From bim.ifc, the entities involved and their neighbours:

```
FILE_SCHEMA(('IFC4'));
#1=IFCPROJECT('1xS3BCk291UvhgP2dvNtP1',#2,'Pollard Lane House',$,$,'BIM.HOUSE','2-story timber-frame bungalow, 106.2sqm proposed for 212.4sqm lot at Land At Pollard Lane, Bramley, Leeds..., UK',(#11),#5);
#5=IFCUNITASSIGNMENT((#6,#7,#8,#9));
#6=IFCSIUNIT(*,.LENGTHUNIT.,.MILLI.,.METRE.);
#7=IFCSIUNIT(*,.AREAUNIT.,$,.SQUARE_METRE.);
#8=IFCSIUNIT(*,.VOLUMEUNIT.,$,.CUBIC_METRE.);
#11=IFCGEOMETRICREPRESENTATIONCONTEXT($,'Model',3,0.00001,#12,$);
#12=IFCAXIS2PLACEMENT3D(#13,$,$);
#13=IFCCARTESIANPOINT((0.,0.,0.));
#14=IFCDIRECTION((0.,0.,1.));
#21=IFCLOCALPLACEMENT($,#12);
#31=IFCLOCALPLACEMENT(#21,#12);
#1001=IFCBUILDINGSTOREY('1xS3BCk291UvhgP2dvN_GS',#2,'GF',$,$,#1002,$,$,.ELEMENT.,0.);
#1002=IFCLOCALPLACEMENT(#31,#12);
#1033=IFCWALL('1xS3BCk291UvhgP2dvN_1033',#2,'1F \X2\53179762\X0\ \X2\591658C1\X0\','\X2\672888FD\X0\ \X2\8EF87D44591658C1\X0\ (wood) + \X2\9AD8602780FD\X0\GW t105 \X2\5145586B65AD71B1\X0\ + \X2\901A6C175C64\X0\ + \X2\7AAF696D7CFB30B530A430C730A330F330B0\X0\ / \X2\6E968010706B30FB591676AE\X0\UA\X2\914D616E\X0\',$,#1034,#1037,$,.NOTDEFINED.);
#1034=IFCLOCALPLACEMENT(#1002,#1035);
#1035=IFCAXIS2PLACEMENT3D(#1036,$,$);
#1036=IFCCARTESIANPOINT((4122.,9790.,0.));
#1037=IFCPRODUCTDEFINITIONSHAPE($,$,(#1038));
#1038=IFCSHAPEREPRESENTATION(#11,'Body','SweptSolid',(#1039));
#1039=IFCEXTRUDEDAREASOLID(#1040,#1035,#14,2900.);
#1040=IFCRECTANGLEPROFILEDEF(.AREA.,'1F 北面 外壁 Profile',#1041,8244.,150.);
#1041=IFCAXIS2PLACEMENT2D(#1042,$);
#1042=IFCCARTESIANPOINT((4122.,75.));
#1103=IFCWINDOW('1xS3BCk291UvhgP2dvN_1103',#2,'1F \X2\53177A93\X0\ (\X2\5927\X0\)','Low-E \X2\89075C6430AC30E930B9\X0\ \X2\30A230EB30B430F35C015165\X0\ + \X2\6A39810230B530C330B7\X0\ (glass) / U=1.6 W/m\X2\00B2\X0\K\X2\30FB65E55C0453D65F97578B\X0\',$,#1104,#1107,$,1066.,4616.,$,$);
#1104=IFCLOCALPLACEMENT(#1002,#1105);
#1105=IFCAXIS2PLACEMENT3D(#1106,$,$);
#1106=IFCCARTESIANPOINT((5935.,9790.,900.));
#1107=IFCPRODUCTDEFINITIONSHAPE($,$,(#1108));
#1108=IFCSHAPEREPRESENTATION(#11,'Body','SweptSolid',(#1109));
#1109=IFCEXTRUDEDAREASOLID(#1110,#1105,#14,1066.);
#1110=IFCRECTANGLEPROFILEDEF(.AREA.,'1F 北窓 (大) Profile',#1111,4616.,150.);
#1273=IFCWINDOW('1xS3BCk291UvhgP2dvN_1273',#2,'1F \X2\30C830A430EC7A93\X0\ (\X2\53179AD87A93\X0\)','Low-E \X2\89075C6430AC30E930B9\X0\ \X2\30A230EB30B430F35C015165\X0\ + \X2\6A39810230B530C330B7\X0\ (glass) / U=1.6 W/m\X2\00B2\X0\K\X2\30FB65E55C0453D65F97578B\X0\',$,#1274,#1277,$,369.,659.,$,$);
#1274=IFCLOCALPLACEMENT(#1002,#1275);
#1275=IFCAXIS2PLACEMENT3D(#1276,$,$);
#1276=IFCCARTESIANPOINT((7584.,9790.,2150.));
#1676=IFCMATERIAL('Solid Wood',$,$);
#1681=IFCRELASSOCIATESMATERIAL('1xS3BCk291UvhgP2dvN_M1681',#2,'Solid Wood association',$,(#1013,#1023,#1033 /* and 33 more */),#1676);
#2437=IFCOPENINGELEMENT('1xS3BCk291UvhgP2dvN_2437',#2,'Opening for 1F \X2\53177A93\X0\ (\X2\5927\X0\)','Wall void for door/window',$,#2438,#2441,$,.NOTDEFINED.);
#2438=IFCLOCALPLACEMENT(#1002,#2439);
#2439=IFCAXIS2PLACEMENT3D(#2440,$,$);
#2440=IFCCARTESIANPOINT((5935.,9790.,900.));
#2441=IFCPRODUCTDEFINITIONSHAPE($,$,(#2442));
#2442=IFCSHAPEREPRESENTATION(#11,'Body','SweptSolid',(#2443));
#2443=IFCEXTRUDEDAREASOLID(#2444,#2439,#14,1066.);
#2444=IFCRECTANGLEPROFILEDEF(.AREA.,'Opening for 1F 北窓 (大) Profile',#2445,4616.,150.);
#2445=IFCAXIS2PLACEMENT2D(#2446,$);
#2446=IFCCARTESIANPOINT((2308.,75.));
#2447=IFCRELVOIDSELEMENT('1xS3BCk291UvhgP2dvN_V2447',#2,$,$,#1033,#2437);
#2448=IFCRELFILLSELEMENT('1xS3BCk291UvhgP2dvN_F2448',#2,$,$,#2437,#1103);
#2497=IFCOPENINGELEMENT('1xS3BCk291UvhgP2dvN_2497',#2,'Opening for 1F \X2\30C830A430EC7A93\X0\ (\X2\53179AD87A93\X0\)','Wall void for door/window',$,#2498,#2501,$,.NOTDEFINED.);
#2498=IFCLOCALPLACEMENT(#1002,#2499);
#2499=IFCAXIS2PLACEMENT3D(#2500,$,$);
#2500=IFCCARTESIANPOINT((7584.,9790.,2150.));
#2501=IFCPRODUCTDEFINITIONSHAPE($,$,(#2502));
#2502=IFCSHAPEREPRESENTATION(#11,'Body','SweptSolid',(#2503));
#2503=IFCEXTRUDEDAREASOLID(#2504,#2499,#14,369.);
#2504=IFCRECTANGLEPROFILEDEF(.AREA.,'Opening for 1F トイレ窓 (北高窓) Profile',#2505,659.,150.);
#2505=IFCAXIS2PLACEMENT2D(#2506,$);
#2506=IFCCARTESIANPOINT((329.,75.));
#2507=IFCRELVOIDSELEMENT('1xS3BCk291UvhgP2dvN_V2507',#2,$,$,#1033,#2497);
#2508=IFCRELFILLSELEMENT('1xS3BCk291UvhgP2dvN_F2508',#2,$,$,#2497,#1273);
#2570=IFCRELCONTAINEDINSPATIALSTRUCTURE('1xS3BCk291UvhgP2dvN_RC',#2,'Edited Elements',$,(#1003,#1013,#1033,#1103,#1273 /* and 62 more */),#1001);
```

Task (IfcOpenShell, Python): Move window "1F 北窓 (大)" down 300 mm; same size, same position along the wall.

```python
import numpy as np
import ifcopenshell
import ifcopenshell.api.geometry
import ifcopenshell.util.placement
import ifcopenshell.util.unit

model = ifcopenshell.open("bim.ifc")
unit_scale = ifcopenshell.util.unit.calculate_unit_scale(model)

window = model.by_guid("1xS3BCk291UvhgP2dvN_1103")
opening = window.FillsVoids[0].RelatingOpeningElement
dz = -0.3 / unit_scale

shift = np.array([0.0, 0.0, dz])
# The window is not placed relative to its opening, so move both.
for product in (opening, window):
    matrix = ifcopenshell.util.placement.get_local_placement(product.ObjectPlacement)
    matrix[:3, 3] += shift
    ifcopenshell.api.geometry.edit_object_placement(model, product=product, matrix=matrix, is_si=False)

print(f"moved by {dz * unit_scale:+.3f} m")

model.write("bim_rev.ifc")
```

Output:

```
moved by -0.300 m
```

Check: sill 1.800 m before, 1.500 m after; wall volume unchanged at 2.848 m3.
